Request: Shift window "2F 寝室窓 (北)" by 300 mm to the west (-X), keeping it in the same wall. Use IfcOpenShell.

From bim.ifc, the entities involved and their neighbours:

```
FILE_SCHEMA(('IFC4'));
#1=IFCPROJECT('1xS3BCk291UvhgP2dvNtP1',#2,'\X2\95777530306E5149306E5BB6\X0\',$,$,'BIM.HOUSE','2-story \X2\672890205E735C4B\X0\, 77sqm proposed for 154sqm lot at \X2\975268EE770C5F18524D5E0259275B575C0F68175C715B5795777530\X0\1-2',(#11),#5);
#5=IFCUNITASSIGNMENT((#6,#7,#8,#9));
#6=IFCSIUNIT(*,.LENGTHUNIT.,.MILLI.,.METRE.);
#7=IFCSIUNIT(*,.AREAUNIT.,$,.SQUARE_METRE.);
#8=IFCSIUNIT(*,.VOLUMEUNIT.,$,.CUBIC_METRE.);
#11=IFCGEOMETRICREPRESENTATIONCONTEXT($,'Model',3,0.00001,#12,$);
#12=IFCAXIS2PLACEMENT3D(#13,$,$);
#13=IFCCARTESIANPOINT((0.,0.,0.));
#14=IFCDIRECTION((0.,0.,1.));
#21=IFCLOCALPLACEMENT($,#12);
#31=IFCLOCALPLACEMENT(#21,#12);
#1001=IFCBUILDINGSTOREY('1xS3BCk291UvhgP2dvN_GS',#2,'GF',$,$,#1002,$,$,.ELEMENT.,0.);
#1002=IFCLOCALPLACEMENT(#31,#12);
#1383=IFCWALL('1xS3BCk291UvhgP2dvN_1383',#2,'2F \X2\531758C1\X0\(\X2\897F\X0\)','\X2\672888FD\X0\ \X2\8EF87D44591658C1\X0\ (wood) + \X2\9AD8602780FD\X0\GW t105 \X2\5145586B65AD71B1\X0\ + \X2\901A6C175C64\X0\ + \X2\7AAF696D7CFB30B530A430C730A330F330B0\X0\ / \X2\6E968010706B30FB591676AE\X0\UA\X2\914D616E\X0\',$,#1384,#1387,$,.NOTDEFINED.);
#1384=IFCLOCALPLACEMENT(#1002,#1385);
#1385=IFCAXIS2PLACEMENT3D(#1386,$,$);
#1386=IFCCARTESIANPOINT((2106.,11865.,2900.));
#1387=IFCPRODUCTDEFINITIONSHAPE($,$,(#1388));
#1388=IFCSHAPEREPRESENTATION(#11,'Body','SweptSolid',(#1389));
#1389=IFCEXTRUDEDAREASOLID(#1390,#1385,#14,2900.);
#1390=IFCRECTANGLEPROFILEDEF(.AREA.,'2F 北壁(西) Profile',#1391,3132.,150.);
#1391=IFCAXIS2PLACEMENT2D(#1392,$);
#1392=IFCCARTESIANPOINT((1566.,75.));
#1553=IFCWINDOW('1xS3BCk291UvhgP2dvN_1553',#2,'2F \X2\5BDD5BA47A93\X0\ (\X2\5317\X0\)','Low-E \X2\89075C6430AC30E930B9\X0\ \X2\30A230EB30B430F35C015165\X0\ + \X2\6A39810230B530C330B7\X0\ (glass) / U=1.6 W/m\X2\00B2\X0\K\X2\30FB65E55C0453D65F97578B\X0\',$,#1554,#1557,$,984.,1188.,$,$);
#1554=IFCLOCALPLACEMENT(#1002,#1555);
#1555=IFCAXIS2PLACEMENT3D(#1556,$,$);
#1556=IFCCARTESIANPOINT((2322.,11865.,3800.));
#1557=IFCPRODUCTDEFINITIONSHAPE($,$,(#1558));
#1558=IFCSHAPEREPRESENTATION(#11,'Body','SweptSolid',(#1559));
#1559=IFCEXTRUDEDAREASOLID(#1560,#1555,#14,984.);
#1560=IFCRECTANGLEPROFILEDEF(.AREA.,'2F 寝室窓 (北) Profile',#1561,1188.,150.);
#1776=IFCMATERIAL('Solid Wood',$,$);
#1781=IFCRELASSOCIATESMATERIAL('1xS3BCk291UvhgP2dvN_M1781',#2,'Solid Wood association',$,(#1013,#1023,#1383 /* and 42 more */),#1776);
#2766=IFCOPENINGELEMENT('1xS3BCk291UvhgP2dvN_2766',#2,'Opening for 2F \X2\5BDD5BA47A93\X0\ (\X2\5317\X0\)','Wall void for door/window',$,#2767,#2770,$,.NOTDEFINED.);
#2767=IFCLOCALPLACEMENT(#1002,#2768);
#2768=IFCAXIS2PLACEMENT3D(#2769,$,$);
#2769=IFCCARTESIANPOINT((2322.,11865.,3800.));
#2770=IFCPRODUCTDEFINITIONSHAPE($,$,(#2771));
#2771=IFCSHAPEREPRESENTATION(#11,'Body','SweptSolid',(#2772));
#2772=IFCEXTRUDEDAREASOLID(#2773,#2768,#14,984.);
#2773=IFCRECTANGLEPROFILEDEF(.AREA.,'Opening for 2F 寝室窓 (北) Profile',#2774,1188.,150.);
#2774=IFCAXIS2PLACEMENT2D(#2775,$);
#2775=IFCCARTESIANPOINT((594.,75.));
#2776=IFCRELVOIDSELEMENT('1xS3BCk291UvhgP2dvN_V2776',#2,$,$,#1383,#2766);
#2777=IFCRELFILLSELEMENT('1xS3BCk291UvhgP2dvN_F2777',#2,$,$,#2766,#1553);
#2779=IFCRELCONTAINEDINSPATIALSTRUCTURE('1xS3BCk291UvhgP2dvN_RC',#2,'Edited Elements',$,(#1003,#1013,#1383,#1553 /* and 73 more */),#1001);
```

```python
import ifcopenshell
import ifcopenshell.api.geometry
import ifcopenshell.util.placement
import ifcopenshell.util.unit

model = ifcopenshell.open("bim.ifc")
unit_scale = ifcopenshell.util.unit.calculate_unit_scale(model)

window = model.by_guid("1xS3BCk291UvhgP2dvN_1553")
opening = window.FillsVoids[0].RelatingOpeningElement
wall = opening.VoidsElements[0].RelatingBuildingElement

wall_matrix = ifcopenshell.util.placement.get_local_placement(wall.ObjectPlacement)
shift = wall_matrix[:3, 0] * -0.3 / unit_scale
before = ifcopenshell.util.placement.get_local_placement(window.ObjectPlacement)[:3, 3].copy()

# The window is not placed relative to its opening, so move both.
for product in (opening, window):
    matrix = ifcopenshell.util.placement.get_local_placement(product.ObjectPlacement)
    matrix[:3, 3] += shift
    ifcopenshell.api.geometry.edit_object_placement(model, product=product, matrix=matrix, is_si=False)

after = ifcopenshell.util.placement.get_local_placement(window.ObjectPlacement)[:3, 3]
print("window moved by", (after - before).round(3) + 0.0)

model.write("bim_updated.ifc")
```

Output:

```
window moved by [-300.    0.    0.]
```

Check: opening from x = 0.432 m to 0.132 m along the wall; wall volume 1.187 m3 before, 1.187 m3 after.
